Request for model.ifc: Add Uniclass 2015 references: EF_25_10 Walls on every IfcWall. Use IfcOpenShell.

First a look at what the model holds.

```python
import ifcopenshell

model = ifcopenshell.open("model.ifc")
print(model.schema)
print("classifications:", [c.Name for c in model.by_type("IfcClassification")])
for ifc_class in ("IfcDoor", "IfcRoof", "IfcStair", "IfcWall", "IfcWindow"):
    print(ifc_class, len(model.by_type(ifc_class)))
```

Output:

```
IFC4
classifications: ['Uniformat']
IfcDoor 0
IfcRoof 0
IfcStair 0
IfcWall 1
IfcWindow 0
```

```python
import ifcopenshell
import ifcopenshell.api.classification

model = ifcopenshell.open("model.ifc")

system = ifcopenshell.api.classification.add_classification(model, classification="Uniclass 2015")

codes = {
    "IfcWall": ("EF_25_10", "Walls"),
}
for ifc_class, (code, name) in codes.items():
    products = model.by_type(ifc_class)
    ifcopenshell.api.classification.add_reference(
        model, products=products, classification=system, identification=code, name=name
    )
    print(code, len(products))

model.write("model_v2.ifc")
```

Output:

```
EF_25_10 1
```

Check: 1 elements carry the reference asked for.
